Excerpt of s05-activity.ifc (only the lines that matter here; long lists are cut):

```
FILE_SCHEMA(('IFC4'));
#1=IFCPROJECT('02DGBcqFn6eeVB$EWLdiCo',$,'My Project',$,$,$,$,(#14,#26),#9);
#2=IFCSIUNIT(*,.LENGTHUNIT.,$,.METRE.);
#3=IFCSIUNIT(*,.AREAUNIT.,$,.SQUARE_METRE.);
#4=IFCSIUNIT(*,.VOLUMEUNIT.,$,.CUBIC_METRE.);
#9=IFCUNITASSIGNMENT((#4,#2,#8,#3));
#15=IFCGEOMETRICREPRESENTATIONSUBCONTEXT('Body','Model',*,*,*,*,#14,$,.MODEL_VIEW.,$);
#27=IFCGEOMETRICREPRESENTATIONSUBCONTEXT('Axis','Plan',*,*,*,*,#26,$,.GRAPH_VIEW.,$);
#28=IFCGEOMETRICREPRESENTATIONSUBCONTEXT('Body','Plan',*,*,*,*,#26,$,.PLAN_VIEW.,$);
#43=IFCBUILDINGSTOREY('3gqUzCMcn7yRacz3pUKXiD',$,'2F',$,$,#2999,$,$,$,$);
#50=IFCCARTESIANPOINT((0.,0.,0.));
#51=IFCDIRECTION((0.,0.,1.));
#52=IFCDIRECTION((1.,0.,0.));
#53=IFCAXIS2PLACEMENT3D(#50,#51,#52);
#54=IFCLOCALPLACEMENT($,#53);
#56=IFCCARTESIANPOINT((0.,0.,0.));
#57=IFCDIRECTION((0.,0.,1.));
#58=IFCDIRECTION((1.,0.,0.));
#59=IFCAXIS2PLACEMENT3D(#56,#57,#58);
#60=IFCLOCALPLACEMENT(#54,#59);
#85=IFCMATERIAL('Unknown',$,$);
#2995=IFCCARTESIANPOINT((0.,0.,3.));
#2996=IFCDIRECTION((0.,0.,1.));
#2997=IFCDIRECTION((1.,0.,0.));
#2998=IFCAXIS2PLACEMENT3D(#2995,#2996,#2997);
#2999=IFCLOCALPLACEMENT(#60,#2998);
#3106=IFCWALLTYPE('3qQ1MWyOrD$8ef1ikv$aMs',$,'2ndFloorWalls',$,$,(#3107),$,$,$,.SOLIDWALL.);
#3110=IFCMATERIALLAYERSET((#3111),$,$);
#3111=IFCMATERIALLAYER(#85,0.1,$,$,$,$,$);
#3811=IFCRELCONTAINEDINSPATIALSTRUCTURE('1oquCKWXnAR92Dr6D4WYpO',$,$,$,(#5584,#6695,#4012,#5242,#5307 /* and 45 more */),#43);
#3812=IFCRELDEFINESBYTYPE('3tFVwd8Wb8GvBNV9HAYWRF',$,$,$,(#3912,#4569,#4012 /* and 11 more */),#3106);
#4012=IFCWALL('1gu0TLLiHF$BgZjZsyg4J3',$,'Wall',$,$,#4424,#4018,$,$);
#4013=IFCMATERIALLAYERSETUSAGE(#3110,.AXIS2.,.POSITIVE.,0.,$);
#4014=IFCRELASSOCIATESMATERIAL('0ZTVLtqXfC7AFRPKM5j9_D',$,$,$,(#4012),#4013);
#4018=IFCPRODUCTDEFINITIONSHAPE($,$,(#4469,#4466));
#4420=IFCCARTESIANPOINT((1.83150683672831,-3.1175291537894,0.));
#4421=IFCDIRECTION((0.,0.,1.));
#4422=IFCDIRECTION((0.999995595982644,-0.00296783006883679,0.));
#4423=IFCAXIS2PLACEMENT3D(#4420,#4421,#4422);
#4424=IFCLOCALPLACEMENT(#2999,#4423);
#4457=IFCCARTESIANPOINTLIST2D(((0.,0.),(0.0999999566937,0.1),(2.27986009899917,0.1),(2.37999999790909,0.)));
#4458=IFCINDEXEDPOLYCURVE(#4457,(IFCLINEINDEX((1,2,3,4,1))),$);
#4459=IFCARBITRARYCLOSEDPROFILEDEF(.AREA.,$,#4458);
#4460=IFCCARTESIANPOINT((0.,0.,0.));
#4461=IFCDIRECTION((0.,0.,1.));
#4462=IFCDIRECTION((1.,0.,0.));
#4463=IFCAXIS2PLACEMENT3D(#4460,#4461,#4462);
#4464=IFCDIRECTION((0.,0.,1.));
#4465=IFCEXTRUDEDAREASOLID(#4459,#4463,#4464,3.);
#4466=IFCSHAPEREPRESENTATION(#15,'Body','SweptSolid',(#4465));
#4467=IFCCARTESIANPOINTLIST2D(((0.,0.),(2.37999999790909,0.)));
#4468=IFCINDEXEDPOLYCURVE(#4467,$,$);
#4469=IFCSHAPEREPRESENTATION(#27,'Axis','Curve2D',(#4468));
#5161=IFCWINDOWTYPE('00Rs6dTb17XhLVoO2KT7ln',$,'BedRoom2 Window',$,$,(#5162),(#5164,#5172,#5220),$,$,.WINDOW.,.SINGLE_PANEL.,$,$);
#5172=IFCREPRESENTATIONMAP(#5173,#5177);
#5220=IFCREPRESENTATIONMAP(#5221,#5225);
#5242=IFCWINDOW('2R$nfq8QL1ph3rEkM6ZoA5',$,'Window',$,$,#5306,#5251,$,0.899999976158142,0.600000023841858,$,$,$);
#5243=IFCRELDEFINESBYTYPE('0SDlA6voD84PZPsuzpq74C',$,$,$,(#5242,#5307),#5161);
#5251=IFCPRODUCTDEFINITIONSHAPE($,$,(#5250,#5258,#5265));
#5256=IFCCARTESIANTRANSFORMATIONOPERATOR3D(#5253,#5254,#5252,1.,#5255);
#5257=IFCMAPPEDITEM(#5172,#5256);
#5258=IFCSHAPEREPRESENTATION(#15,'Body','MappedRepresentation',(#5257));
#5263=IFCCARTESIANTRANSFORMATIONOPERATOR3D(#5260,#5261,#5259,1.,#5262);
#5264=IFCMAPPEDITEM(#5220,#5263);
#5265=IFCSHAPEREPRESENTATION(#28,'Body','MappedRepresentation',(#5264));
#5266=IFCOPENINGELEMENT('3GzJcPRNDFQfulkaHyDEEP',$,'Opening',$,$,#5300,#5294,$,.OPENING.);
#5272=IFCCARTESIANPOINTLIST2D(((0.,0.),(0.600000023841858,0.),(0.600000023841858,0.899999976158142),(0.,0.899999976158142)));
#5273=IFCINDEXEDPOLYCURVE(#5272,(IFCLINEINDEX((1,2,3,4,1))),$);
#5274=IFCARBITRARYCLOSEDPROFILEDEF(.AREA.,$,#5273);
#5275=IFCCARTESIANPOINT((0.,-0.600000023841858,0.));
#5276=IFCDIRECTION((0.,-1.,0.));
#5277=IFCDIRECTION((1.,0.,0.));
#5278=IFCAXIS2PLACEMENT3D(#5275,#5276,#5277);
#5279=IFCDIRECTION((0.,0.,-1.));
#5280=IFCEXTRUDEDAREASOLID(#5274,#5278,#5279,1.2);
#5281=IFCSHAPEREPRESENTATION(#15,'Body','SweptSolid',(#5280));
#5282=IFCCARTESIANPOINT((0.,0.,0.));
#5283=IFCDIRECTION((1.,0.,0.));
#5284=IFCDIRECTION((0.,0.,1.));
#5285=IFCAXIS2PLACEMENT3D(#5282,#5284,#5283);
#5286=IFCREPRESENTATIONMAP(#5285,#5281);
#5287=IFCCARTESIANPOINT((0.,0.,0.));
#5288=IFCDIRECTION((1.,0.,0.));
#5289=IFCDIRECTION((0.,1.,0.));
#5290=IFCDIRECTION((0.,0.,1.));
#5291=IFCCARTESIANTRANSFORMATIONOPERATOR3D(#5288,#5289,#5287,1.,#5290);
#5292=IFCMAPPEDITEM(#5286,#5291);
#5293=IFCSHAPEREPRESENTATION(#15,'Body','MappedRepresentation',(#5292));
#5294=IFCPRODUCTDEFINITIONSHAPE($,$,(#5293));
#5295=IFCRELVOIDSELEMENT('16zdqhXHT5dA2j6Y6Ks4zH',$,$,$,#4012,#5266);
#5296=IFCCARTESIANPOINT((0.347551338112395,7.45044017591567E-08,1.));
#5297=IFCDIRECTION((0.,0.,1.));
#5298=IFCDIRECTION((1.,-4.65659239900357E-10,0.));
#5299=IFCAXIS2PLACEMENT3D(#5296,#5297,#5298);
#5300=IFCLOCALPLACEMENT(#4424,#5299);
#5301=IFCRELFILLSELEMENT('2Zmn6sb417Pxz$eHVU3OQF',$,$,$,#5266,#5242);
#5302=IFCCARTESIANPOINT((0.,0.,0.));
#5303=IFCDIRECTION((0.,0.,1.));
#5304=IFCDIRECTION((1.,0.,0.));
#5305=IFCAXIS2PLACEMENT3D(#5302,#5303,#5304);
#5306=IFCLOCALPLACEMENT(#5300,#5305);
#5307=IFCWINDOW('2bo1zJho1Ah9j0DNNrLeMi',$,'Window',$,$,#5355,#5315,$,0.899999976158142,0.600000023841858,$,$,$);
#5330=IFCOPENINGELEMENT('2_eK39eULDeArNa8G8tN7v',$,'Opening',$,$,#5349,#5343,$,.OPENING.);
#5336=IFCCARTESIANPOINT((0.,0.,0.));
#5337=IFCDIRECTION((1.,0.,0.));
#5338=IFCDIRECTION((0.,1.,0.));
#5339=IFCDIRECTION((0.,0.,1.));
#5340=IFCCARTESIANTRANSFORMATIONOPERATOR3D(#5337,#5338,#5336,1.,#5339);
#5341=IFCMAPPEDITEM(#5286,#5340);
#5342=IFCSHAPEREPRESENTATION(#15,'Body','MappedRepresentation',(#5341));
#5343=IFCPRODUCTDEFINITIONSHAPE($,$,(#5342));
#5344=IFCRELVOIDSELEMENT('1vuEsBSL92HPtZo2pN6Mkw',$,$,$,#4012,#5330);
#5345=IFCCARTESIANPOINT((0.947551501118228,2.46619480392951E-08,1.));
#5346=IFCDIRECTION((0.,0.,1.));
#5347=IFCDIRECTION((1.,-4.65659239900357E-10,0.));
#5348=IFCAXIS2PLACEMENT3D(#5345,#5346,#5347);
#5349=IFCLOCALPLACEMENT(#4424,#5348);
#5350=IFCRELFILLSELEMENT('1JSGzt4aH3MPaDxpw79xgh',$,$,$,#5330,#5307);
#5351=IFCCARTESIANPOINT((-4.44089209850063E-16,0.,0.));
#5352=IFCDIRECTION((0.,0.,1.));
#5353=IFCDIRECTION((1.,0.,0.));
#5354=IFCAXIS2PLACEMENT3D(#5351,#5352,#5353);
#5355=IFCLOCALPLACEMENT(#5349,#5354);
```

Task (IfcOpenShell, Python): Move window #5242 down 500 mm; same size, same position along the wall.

```python
import numpy as np
import ifcopenshell
import ifcopenshell.api.geometry
import ifcopenshell.util.placement
import ifcopenshell.util.unit

model = ifcopenshell.open("s05-activity.ifc")
unit_scale = ifcopenshell.util.unit.calculate_unit_scale(model)

window = model.by_guid("2R$nfq8QL1ph3rEkM6ZoA5")
opening = window.FillsVoids[0].RelatingOpeningElement
dz = -0.5

shift = np.array([0.0, 0.0, dz])
# The window is placed relative to its opening, so it follows when the opening moves.
matrix = ifcopenshell.util.placement.get_local_placement(opening.ObjectPlacement)
matrix[:3, 3] += shift
ifcopenshell.api.geometry.edit_object_placement(
    model, product=opening, matrix=matrix, is_si=False, should_transform_children=True
)

print(f"moved by {dz * unit_scale:+.3f} m")

model.write("s05-activity_edited.ifc")
```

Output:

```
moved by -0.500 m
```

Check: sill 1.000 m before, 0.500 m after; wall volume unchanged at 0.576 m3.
